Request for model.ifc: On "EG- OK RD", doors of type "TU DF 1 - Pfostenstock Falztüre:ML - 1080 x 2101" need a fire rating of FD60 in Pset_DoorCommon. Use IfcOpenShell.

First a look at what the model holds.

```python
import ifcopenshell
import ifcopenshell.util.element

model = ifcopenshell.open("model.ifc")
print(model.schema)
storey = next(s for s in model.by_type("IfcBuildingStorey") if s.Name == "EG- OK RD")
doors = [e for e in ifcopenshell.util.element.get_decomposition(storey) if e.is_a("IfcDoor")]
seen = {}
for e in doors:
    element_type = ifcopenshell.util.element.get_type(e)
    key = (element_type.Name if element_type != e and element_type else None, ifcopenshell.util.element.get_pset(e, "Pset_DoorCommon", "FireRating"))
    seen[key] = seen.get(key, 0) + 1
for (name, value), count in sorted(seen.items(), key=str):
    print(count, "x", name, "|", value)
```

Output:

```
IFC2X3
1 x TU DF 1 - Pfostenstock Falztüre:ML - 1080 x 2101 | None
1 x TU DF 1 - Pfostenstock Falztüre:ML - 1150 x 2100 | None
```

```python
import ifcopenshell
import ifcopenshell.api.pset
import ifcopenshell.util.element

model = ifcopenshell.open("model.ifc")

storey = next(s for s in model.by_type("IfcBuildingStorey") if s.Name == "EG- OK RD")
doors = [e for e in ifcopenshell.util.element.get_decomposition(storey) if e.is_a("IfcDoor")]

count = 0
for e in doors:
    element_type = ifcopenshell.util.element.get_type(e)
    if element_type in (None, e) or element_type.Name != "TU DF 1 - Pfostenstock Falztüre:ML - 1080 x 2101":
        continue
    # add_pset returns the element's existing set when there is one.
    pset = ifcopenshell.api.pset.add_pset(model, product=e, name="Pset_DoorCommon")
    ifcopenshell.api.pset.edit_pset(model, pset=pset, properties={"FireRating": "FD60"})
    count += 1

print(count, "doors updated")

model.write("model_v2.ifc")
```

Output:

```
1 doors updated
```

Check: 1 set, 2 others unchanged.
